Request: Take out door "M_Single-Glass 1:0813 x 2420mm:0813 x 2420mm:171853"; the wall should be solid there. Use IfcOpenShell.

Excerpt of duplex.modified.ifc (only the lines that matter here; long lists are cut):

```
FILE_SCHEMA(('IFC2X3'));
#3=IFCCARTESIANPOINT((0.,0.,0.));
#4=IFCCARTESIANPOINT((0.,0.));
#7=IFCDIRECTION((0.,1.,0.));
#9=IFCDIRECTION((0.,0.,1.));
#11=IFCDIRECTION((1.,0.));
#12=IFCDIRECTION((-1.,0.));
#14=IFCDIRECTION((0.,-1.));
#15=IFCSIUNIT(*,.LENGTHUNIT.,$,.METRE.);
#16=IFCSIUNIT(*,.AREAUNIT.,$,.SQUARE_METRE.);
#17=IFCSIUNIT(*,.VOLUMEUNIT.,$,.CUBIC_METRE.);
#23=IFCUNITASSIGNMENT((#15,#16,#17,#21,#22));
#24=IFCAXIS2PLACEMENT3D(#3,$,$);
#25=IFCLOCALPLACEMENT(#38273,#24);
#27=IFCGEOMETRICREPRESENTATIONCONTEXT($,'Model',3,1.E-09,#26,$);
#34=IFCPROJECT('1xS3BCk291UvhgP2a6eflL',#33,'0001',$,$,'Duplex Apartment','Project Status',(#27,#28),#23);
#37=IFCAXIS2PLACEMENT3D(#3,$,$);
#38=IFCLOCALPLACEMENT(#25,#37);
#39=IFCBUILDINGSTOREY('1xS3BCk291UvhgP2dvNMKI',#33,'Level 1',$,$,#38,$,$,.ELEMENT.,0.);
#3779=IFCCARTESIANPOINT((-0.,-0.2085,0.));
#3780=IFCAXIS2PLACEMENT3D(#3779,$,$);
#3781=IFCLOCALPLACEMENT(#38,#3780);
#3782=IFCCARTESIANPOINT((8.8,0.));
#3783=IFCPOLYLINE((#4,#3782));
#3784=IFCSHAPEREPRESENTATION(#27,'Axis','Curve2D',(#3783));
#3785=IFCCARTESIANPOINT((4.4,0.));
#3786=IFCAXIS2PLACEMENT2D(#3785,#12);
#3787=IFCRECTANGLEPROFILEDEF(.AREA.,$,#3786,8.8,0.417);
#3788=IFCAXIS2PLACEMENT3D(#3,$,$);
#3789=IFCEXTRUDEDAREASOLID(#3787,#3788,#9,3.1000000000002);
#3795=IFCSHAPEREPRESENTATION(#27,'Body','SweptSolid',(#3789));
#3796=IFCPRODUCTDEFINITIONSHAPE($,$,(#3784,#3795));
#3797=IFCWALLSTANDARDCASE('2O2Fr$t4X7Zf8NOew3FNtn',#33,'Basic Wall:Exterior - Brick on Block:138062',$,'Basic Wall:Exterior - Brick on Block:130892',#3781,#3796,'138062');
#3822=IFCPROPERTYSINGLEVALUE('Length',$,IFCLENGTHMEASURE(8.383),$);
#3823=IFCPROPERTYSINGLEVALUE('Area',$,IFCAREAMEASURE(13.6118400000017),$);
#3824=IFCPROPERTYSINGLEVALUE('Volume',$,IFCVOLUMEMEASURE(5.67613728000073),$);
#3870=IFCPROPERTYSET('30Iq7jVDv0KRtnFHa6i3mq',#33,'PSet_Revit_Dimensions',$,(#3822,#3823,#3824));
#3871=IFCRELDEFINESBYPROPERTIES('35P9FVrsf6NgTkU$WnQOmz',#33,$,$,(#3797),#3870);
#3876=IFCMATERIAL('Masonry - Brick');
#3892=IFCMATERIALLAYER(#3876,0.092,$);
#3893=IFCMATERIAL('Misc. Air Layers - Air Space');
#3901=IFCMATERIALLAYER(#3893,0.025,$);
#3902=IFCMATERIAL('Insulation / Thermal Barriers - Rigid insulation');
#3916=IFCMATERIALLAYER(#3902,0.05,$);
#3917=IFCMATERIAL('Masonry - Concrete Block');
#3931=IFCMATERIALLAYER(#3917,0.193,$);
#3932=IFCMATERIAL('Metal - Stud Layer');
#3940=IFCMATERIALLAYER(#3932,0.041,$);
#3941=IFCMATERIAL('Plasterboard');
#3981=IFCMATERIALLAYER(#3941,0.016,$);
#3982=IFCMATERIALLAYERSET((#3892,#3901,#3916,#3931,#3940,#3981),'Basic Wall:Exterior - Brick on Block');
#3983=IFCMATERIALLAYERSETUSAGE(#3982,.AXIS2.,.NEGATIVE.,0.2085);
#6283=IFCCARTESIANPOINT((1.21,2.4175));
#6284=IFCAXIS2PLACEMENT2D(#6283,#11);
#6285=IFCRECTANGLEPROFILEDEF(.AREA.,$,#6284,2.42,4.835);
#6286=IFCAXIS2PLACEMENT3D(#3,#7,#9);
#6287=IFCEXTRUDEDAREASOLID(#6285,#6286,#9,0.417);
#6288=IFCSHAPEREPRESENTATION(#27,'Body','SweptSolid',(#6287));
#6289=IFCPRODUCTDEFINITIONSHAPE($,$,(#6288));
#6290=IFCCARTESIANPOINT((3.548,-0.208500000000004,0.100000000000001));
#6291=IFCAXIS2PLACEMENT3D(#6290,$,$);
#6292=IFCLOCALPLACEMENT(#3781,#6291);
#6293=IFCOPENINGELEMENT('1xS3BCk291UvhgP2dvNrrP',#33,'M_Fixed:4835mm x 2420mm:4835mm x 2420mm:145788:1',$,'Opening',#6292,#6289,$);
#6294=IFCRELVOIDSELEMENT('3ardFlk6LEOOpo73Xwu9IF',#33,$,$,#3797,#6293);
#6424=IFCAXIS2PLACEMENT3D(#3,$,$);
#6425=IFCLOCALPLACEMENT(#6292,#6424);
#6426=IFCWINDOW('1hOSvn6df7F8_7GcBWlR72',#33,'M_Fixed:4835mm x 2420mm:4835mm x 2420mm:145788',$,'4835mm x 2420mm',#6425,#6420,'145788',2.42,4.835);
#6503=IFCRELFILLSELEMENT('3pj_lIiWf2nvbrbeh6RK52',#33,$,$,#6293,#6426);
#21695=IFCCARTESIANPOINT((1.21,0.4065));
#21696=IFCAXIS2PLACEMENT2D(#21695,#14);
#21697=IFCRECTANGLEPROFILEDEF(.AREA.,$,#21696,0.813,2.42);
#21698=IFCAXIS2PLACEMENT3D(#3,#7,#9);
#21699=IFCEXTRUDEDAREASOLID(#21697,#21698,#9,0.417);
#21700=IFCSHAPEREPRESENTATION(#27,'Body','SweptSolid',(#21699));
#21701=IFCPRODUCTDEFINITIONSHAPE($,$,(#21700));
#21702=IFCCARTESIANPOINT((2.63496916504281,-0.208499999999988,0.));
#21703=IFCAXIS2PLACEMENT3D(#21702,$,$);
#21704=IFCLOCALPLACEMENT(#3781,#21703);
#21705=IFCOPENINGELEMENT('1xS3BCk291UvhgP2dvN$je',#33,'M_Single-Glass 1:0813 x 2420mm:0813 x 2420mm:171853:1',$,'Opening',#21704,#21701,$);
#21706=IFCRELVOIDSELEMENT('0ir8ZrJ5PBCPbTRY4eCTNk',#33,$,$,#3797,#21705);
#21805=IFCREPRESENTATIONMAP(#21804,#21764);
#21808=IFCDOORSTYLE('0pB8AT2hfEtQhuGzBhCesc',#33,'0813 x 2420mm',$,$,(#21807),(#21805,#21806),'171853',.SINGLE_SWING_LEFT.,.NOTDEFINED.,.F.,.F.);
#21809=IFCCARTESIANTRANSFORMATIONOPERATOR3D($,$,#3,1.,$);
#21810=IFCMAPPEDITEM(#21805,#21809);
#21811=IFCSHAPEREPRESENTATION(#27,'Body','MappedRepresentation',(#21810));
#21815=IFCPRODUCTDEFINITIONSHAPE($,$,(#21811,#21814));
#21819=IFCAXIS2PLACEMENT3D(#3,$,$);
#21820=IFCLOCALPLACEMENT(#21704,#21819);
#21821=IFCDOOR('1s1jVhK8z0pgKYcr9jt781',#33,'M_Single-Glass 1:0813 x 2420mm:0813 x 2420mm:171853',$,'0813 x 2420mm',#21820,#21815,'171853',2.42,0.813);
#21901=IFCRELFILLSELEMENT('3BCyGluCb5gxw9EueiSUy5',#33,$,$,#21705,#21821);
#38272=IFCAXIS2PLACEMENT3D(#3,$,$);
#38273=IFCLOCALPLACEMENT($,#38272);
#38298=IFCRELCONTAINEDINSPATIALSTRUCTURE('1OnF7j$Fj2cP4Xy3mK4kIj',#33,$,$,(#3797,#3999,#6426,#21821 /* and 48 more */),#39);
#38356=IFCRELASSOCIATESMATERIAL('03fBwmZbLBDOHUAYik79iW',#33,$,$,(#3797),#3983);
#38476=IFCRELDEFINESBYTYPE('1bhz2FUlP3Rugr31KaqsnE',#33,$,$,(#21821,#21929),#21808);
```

```python
import ifcopenshell
import ifcopenshell.api.feature
import ifcopenshell.api.pset
import ifcopenshell.api.root
import ifcopenshell.geom
import ifcopenshell.util.element
import ifcopenshell.util.shape
import ifcopenshell.util.unit

model = ifcopenshell.open("duplex.modified.ifc")
area_scale = ifcopenshell.util.unit.calculate_unit_scale(model, "AREAUNIT")
volume_scale = ifcopenshell.util.unit.calculate_unit_scale(model, "VOLUMEUNIT")
settings = ifcopenshell.geom.settings()


def volume(element):
    """Net volume in cubic metres, openings subtracted."""
    shape = ifcopenshell.geom.create_shape(settings, element)
    return ifcopenshell.util.shape.get_volume(shape.geometry)


door = model.by_guid("1s1jVhK8z0pgKYcr9jt781")
opening = door.FillsVoids[0].RelatingOpeningElement
wall = opening.VoidsElements[0].RelatingBuildingElement
before = volume(wall)

ifcopenshell.api.root.remove_product(model, product=door)
ifcopenshell.api.feature.remove_feature(model, feature=opening)

after = volume(wall)
thickness = 0.417  # wall thickness in metres

# Update the wall's stored quantities.
pset = model.by_id(ifcopenshell.util.element.get_pset(wall, "PSet_Revit_Dimensions", should_inherit=False)["id"])
ifcopenshell.api.pset.edit_pset(model, pset=pset, properties={
    "Area": model.create_entity("IfcAreaMeasure", after / thickness / area_scale),
    "Volume": model.create_entity("IfcVolumeMeasure", after / volume_scale),
})

print(f"wall volume {before:.3f} -> {after:.3f} m3")

model.write("duplex.modified_rev.ifc")
```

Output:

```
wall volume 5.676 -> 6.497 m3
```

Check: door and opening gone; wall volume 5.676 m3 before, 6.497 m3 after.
